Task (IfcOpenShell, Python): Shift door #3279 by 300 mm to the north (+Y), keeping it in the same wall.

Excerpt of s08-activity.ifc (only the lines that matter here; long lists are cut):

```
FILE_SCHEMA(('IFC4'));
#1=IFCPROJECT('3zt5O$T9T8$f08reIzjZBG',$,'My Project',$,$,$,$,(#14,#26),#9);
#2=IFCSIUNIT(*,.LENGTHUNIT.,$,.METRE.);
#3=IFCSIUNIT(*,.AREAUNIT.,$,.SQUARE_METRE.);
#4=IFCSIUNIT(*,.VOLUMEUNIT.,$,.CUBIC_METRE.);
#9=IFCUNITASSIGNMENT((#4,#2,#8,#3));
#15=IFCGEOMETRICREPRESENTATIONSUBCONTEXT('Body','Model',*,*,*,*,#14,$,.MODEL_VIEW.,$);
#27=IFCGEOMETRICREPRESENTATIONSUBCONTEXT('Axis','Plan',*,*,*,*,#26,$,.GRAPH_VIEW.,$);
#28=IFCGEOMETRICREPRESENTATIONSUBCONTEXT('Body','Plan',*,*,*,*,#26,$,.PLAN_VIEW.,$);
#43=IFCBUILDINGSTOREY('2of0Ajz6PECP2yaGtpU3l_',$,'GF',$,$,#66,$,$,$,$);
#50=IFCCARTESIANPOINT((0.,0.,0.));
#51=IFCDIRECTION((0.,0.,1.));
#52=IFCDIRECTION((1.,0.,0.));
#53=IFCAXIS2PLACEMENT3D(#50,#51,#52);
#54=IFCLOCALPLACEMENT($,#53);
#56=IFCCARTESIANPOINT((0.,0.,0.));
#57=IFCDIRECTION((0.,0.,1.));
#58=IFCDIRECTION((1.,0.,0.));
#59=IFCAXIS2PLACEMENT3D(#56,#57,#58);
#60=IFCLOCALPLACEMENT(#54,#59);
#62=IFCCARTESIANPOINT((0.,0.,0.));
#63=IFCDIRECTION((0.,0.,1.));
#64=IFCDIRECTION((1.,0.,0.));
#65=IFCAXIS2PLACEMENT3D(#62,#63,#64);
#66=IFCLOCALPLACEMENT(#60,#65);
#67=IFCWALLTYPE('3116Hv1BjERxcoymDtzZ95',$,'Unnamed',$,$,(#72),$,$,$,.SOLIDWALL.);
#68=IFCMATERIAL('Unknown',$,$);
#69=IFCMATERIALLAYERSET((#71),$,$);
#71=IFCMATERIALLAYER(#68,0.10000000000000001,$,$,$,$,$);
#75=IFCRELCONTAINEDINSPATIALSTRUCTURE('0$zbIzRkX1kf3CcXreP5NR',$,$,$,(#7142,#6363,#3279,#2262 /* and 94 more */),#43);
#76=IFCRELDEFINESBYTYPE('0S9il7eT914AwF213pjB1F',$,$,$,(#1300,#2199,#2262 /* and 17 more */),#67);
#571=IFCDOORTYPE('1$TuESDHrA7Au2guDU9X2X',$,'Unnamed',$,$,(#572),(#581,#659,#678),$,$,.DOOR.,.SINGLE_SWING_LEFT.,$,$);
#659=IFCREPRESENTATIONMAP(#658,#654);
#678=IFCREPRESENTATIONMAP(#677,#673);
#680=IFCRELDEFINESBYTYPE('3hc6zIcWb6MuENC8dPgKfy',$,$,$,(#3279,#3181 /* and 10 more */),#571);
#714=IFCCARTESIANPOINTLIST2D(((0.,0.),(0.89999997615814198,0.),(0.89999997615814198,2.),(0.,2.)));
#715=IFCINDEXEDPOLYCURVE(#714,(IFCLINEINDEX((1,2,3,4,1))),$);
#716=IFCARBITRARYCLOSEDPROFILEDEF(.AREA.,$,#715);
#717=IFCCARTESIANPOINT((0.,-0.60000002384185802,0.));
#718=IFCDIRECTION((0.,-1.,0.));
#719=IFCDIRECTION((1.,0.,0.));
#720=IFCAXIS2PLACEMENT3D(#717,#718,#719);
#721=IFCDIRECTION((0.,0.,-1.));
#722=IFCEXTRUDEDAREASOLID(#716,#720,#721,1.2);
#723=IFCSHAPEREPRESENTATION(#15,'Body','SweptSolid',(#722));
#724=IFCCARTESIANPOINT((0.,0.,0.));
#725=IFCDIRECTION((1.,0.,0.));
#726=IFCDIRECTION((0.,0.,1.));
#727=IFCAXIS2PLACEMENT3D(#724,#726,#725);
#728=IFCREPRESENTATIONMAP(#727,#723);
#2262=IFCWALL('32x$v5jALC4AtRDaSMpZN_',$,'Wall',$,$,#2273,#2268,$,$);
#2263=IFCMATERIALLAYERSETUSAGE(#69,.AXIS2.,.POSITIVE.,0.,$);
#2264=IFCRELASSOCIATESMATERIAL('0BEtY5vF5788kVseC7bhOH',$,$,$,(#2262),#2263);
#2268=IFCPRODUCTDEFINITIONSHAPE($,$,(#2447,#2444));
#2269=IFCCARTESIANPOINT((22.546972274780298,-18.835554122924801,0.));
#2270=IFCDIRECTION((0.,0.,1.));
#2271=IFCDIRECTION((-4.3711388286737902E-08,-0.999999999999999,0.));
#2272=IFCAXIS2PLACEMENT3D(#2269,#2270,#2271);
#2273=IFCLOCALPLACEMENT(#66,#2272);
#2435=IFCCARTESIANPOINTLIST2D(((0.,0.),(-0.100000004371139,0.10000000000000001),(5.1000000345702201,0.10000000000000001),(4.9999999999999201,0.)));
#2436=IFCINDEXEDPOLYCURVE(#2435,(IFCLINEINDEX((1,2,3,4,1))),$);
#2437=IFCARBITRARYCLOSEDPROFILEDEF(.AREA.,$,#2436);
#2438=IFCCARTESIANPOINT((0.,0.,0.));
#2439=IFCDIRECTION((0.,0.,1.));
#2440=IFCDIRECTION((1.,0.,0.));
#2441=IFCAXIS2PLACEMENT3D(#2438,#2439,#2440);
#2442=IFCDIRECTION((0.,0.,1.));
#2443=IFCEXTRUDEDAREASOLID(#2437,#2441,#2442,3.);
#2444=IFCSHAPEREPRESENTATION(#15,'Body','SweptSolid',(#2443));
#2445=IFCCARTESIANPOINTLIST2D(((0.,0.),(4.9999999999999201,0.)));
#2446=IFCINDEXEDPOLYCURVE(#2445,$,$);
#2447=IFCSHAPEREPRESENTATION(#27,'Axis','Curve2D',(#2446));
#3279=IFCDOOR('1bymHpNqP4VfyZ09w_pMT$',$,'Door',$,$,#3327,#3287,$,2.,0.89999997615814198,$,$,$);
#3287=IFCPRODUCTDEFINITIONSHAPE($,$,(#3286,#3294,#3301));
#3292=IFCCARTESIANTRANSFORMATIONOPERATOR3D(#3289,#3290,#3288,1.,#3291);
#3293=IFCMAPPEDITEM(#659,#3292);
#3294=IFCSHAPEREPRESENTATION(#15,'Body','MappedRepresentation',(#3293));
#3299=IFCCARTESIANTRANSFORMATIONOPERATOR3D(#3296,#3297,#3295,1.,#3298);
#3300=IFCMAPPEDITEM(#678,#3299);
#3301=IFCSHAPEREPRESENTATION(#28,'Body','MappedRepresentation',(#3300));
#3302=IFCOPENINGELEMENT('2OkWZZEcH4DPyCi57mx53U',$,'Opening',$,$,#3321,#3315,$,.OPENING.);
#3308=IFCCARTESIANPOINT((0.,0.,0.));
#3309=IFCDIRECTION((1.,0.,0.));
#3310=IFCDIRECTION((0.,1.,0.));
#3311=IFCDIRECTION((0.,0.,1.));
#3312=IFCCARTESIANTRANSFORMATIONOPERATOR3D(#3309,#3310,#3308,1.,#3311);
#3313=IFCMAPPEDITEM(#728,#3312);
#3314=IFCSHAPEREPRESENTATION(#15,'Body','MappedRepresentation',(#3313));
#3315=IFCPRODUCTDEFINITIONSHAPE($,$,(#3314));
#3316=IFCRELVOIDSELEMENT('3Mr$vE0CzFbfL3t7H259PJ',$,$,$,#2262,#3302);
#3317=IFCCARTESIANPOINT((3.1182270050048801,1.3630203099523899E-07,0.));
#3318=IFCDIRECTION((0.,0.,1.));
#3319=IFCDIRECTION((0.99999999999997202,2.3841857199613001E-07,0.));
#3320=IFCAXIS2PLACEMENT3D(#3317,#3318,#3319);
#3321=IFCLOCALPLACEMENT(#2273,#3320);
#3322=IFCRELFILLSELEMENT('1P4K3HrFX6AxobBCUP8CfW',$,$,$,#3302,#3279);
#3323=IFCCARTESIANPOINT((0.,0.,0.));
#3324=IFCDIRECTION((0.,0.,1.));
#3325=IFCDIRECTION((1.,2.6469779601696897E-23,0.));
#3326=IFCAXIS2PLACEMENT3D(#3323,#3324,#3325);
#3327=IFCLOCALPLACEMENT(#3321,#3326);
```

```python
import ifcopenshell
import ifcopenshell.api.geometry
import ifcopenshell.util.placement

model = ifcopenshell.open("s08-activity.ifc")

door = model.by_id(3279)
opening = door.FillsVoids[0].RelatingOpeningElement
wall = opening.VoidsElements[0].RelatingBuildingElement

wall_matrix = ifcopenshell.util.placement.get_local_placement(wall.ObjectPlacement)
shift = wall_matrix[:3, 0] * -0.3
before = ifcopenshell.util.placement.get_local_placement(door.ObjectPlacement)[:3, 3].copy()

# The door is placed relative to its opening, so it follows when the opening moves.
matrix = ifcopenshell.util.placement.get_local_placement(opening.ObjectPlacement)
matrix[:3, 3] += shift
ifcopenshell.api.geometry.edit_object_placement(
    model, product=opening, matrix=matrix, is_si=False, should_transform_children=True
)

after = ifcopenshell.util.placement.get_local_placement(door.ObjectPlacement)[:3, 3]
print("door moved by", (after - before).round(3) + 0.0)

model.write("s08-activity_rev.ifc")
```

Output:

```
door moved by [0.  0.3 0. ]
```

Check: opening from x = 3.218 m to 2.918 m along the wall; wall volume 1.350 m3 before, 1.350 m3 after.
